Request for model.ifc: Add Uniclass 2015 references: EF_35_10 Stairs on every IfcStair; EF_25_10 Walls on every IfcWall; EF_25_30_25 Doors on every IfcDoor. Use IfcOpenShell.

First a look at what the model holds.

```python
import ifcopenshell

model = ifcopenshell.open("model.ifc")
print(model.schema)
print("classifications:", [c.Name for c in model.by_type("IfcClassification")])
for ifc_class in ("IfcDoor", "IfcRoof", "IfcStair", "IfcWall", "IfcWindow"):
    print(ifc_class, len(model.by_type(ifc_class)))
```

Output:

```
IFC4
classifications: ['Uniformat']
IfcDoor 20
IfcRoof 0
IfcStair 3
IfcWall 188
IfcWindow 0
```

```python
import ifcopenshell
import ifcopenshell.api.classification

model = ifcopenshell.open("model.ifc")

system = ifcopenshell.api.classification.add_classification(model, classification="Uniclass 2015")

codes = {
    "IfcStair": ("EF_35_10", "Stairs"),
    "IfcWall": ("EF_25_10", "Walls"),
    "IfcDoor": ("EF_25_30_25", "Doors"),
}
for ifc_class, (code, name) in codes.items():
    products = model.by_type(ifc_class)
    ifcopenshell.api.classification.add_reference(
        model, products=products, classification=system, identification=code, name=name
    )
    print(code, len(products))

model.write("model-out.ifc")
```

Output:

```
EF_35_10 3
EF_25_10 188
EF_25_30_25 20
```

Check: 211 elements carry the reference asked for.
